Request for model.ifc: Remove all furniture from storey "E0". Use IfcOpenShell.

First a look at what the model holds.

```python
import ifcopenshell
import ifcopenshell.util.element

model = ifcopenshell.open("model.ifc")
print(model.schema)
storey = next(s for s in model.by_type("IfcBuildingStorey") if s.Name == "E0")
furniture = [e for e in ifcopenshell.util.element.get_decomposition(storey) if e.is_a("IfcFurnishingElement")]
seen = {}
for e in furniture:
    element_type = ifcopenshell.util.element.get_type(e)
    name = element_type.Name if element_type not in (None, e) else None
    seen[name] = seen.get(name, 0) + 1
for name, count in sorted(seen.items(), key=str):
    print(count, "x", name)
```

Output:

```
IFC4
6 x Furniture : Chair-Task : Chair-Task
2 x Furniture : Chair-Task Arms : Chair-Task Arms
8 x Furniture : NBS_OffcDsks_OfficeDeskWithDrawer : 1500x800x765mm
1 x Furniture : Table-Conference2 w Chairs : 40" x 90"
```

```python
import ifcopenshell
import ifcopenshell.api.root
import ifcopenshell.util.element

model = ifcopenshell.open("model.ifc")

storey = next(s for s in model.by_type("IfcBuildingStorey") if s.Name == "E0")
furniture = [e for e in ifcopenshell.util.element.get_decomposition(storey) if e.is_a("IfcFurnishingElement")]

for e in furniture:
    ifcopenshell.api.root.remove_product(model, product=e)
print(len(furniture), "removed")

model.write("model_v2.ifc")
```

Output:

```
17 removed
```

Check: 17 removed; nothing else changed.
